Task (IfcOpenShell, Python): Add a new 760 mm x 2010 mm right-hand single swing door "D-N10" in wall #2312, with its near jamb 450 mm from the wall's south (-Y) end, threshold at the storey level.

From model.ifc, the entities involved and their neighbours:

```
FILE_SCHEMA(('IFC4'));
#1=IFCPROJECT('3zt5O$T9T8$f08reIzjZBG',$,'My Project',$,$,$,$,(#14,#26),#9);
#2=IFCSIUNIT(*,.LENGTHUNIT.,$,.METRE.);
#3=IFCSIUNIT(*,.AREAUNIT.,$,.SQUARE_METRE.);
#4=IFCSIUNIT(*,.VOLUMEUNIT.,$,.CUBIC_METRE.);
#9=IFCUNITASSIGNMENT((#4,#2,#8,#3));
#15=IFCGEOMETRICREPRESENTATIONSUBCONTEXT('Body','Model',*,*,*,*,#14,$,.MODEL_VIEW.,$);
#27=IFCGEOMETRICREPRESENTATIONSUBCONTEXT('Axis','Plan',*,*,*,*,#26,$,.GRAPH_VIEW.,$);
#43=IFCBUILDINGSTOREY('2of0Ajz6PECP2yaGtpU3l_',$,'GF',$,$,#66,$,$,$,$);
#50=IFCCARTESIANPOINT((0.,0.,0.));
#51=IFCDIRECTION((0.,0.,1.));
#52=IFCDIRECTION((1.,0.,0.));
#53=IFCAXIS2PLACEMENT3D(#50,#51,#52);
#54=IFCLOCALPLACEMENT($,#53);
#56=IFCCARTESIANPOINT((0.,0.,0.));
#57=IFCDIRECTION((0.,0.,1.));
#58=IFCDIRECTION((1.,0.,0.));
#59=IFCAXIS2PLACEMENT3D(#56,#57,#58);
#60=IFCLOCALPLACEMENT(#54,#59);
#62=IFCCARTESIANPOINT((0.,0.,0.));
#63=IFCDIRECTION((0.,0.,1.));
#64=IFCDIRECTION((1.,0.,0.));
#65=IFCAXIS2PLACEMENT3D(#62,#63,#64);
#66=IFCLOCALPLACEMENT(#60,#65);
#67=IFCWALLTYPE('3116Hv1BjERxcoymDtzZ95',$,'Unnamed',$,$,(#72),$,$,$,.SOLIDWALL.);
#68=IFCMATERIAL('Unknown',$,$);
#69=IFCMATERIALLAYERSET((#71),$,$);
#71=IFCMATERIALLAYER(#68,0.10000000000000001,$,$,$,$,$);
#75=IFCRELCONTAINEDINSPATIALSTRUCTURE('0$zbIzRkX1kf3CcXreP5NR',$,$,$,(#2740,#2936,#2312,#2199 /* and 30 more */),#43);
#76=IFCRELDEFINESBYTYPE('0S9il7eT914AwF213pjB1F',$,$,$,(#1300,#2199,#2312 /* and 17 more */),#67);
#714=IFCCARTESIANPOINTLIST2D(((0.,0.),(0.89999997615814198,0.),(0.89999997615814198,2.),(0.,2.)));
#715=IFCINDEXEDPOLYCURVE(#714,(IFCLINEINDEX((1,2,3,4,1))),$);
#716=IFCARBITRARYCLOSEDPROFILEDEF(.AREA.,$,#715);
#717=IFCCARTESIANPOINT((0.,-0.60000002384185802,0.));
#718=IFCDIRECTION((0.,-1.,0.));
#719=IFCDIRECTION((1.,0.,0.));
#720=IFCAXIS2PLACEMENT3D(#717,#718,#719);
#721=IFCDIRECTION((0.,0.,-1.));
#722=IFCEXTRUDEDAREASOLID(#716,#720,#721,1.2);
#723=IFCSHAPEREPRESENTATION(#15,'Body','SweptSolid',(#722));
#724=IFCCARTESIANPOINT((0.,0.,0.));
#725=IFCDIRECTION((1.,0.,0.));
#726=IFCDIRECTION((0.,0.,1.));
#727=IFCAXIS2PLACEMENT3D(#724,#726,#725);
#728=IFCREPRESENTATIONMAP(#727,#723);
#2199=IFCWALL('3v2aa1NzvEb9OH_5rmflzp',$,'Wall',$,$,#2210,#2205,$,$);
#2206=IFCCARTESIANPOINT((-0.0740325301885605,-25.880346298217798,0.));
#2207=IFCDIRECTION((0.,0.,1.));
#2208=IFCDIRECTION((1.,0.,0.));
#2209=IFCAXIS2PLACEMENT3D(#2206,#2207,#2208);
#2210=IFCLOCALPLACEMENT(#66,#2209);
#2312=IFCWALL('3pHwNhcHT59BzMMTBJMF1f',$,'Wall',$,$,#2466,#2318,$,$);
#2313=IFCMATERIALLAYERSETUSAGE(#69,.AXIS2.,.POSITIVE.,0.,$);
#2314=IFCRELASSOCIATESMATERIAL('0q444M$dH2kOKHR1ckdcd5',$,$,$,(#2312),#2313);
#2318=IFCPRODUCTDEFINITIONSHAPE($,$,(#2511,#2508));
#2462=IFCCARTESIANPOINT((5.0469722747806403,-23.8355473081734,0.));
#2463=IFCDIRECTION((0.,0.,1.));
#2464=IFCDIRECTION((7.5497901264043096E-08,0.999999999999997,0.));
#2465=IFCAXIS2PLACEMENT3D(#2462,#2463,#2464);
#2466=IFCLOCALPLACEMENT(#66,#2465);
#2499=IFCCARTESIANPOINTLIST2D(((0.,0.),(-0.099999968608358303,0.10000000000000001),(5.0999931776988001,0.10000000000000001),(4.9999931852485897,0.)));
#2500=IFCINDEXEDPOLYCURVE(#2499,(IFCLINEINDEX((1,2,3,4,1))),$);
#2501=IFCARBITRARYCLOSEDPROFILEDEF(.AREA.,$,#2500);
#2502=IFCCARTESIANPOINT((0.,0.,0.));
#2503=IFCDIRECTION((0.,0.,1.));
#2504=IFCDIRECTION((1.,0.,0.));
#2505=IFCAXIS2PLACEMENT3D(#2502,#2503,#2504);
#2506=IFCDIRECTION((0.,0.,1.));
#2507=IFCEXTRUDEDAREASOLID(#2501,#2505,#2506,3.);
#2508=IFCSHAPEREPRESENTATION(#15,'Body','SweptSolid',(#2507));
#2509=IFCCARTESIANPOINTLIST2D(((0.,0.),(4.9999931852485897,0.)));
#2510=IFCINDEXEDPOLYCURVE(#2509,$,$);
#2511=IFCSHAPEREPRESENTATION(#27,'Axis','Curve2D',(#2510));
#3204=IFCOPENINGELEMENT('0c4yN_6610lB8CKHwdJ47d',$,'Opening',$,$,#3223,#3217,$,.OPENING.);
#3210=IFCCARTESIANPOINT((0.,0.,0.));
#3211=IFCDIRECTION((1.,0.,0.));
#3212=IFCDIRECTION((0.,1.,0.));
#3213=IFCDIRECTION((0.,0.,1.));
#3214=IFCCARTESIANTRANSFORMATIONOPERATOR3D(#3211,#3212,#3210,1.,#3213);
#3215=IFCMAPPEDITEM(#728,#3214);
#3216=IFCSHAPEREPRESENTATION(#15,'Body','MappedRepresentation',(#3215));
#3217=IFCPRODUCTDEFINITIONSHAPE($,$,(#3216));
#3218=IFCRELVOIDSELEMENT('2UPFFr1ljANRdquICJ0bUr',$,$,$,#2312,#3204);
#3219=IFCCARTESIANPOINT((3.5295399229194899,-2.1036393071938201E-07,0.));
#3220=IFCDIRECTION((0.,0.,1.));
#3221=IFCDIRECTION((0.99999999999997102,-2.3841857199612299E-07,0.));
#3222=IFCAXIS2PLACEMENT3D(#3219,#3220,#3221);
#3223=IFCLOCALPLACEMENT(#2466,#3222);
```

```python
import numpy as np
import ifcopenshell
import ifcopenshell.api.feature
import ifcopenshell.api.geometry
import ifcopenshell.api.root
import ifcopenshell.api.spatial
import ifcopenshell.geom
import ifcopenshell.util.element
import ifcopenshell.util.placement
import ifcopenshell.util.representation
import ifcopenshell.util.shape
import ifcopenshell.util.unit

model = ifcopenshell.open("model.ifc")
unit_scale = ifcopenshell.util.unit.calculate_unit_scale(model)
settings = ifcopenshell.geom.settings()


def volume(element):
    """Net volume in cubic metres, openings subtracted."""
    shape = ifcopenshell.geom.create_shape(settings, element)
    return ifcopenshell.util.shape.get_volume(shape.geometry)


wall = model.by_guid("3pHwNhcHT59BzMMTBJMF1f")
storey = ifcopenshell.util.element.get_container(wall, ifc_class="IfcBuildingStorey")
context = ifcopenshell.util.representation.get_context(model, "Model", "Body", "MODEL_VIEW")
before = volume(wall)

width, height, from_end, sill = 0.76, 2.01, 0.45, 0.0  # metres

# The wall runs along its own X axis, and the end named is its -X end.
wall_shape = ifcopenshell.geom.create_shape(settings, wall)
x, y, z = ifcopenshell.util.shape.get_vertices(wall_shape.geometry).T
start = x.min() + from_end
face, thickness = float(y.min()), float(y.max() - y.min())
wall_matrix = ifcopenshell.util.placement.get_local_placement(wall.ObjectPlacement)
level = ifcopenshell.util.placement.get_local_placement(storey.ObjectPlacement)[2, 3]


def in_wall(x, y):
    """Placement at x, y metres in the wall's axes, at sill height."""
    matrix = wall_matrix.copy()
    matrix[:, 3] = wall_matrix @ np.array([x / unit_scale, y / unit_scale, 0.0, 1.0])
    matrix[2, 3] = level + sill / unit_scale
    return matrix


# Opening: a box that overshoots both wall faces by 50 mm.
opening = ifcopenshell.api.root.create_entity(model, ifc_class="IfcOpeningElement", predefined_type="OPENING")
box = ifcopenshell.api.geometry.add_wall_representation(
    model, context=context, length=width, height=height, thickness=thickness + 0.1
)
ifcopenshell.api.geometry.assign_representation(model, product=opening, representation=box)
ifcopenshell.api.geometry.edit_object_placement(model, product=opening, matrix=in_wall(start, face - 0.05), is_si=False)
ifcopenshell.api.feature.add_feature(model, feature=opening, element=wall)

door = ifcopenshell.api.root.create_entity(model, ifc_class="IfcDoor", name="D-N10", predefined_type="DOOR")
door.OverallWidth, door.OverallHeight = width / unit_scale, height / unit_scale
door.OperationType = "SINGLE_SWING_RIGHT"
body = ifcopenshell.api.geometry.add_door_representation(
    model,
    context=context,
    overall_width=door.OverallWidth,
    overall_height=door.OverallHeight,
    operation_type="SINGLE_SWING_RIGHT",
    lining_properties={"LiningDepth": thickness / unit_scale, "ThresholdDepth": thickness / unit_scale},
)
ifcopenshell.api.geometry.assign_representation(model, product=door, representation=body)
ifcopenshell.api.spatial.assign_container(model, products=[door], relating_structure=storey)
ifcopenshell.api.feature.add_filling(model, opening=opening, element=door)

# The lining spans the wall, so the door starts at the wall face.
ifcopenshell.api.geometry.edit_object_placement(model, product=door, matrix=in_wall(start, face), is_si=False)

after = volume(wall)

print(f"wall volume {before:.3f} -> {after:.3f} m3")

model.write("model_updated.ifc")
```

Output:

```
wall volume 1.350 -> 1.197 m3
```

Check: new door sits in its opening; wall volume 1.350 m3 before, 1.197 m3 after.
